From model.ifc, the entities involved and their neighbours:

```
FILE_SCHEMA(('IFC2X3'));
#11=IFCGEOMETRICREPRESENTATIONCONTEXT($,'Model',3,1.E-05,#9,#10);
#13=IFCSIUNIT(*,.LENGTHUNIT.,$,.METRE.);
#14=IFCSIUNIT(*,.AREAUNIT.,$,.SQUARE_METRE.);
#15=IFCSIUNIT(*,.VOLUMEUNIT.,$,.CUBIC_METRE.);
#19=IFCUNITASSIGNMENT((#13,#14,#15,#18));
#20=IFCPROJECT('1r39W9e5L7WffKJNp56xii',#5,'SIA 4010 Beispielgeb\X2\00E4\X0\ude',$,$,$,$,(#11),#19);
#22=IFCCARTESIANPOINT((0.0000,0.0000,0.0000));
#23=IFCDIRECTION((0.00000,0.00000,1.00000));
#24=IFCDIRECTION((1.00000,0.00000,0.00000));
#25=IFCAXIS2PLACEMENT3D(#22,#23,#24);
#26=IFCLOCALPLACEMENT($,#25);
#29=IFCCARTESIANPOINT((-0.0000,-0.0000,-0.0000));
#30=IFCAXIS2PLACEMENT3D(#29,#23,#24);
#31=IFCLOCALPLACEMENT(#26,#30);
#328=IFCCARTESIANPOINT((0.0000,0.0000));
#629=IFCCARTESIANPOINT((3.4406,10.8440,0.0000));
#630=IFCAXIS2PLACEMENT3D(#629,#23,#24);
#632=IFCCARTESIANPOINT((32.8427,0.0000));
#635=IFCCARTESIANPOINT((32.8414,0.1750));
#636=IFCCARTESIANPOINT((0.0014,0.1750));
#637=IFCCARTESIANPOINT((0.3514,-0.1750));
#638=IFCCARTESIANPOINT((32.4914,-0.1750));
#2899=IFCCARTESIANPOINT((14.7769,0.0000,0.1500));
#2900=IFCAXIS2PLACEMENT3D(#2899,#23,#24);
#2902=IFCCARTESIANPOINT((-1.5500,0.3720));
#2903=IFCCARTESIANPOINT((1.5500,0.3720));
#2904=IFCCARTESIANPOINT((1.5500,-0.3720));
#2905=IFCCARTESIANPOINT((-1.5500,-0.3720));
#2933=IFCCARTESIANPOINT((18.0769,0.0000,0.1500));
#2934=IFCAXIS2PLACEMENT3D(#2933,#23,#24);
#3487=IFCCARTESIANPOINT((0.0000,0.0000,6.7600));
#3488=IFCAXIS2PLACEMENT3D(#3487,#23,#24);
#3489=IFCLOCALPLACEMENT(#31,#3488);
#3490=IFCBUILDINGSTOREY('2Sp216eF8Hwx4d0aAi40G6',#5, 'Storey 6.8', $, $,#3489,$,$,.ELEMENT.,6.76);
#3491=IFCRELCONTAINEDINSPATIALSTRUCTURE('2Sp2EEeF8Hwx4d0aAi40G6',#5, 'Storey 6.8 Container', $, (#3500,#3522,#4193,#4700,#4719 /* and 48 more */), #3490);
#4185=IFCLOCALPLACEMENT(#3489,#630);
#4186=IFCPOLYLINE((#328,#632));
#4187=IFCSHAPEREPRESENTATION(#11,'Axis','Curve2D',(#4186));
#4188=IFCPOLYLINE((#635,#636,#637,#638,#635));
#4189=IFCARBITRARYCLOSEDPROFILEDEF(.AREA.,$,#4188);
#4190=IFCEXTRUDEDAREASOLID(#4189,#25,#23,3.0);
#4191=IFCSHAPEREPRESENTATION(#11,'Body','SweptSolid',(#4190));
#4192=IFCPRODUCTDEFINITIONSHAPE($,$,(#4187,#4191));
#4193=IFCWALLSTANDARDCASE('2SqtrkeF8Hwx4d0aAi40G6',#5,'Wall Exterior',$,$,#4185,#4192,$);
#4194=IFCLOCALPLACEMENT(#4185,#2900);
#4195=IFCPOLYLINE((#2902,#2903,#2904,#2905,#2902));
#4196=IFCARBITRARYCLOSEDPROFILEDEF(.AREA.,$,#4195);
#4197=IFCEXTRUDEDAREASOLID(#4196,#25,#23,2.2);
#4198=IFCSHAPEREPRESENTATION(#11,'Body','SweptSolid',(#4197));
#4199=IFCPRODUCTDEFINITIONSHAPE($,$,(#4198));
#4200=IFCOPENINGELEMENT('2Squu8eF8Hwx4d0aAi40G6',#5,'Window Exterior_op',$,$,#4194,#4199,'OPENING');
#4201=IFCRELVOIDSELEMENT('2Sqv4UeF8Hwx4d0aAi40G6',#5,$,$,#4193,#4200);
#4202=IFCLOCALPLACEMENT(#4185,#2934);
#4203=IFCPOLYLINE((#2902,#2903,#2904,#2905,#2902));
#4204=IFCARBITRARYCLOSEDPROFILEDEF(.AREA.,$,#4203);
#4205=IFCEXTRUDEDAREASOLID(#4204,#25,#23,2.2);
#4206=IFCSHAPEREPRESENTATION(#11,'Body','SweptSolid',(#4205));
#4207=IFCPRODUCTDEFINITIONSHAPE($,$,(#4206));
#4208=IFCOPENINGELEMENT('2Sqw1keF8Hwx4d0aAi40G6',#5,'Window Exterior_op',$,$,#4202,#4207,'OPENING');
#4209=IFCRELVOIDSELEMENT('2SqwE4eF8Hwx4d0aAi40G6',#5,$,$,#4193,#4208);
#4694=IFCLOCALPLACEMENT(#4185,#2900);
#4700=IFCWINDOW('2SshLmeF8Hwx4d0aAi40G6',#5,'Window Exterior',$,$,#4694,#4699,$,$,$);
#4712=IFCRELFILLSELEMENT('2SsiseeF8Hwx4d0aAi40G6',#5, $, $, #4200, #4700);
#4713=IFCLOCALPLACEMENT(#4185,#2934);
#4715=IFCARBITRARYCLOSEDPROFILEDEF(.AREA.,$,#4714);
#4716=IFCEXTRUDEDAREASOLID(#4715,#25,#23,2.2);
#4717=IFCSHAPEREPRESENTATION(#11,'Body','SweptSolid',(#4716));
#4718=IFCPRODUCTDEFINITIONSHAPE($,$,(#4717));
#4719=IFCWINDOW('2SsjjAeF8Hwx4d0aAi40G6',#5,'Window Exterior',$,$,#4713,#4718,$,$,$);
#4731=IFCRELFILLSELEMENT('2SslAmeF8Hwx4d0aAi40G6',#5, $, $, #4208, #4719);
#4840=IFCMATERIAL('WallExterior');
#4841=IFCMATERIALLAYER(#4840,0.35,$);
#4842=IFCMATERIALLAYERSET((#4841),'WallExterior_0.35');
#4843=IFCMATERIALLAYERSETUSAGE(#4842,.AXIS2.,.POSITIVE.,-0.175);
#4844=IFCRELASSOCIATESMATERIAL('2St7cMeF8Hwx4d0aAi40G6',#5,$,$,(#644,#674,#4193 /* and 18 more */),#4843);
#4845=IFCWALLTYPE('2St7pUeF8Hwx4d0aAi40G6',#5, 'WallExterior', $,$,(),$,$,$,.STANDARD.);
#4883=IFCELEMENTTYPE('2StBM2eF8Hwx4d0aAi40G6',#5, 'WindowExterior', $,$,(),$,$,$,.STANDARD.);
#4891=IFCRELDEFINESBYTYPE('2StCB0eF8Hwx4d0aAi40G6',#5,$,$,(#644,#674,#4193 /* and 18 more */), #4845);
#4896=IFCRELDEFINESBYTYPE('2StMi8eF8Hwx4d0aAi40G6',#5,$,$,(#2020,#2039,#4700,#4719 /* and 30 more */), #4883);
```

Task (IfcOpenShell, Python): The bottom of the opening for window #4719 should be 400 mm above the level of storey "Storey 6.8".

```python
import numpy as np
import ifcopenshell
import ifcopenshell.api.geometry
import ifcopenshell.geom
import ifcopenshell.util.element
import ifcopenshell.util.placement
import ifcopenshell.util.shape
import ifcopenshell.util.unit

model = ifcopenshell.open("model.ifc")
unit_scale = ifcopenshell.util.unit.calculate_unit_scale(model)

window = model.by_guid("2SsjjAeF8Hwx4d0aAi40G6")
opening = window.FillsVoids[0].RelatingOpeningElement
storey = ifcopenshell.util.element.get_container(window, ifc_class="IfcBuildingStorey")
level = ifcopenshell.util.placement.get_local_placement(storey.ObjectPlacement)[2, 3]

# The opening's origin need not be at the sill, so measure its lowest point.
shape = ifcopenshell.geom.create_shape(ifcopenshell.geom.settings(), opening)
bottom = ifcopenshell.util.shape.get_shape_bottom_elevation(shape, shape.geometry) / unit_scale
dz = level + 0.4 / unit_scale - bottom

shift = np.array([0.0, 0.0, dz])
# The window is not placed relative to its opening, so move both.
for product in (opening, window):
    matrix = ifcopenshell.util.placement.get_local_placement(product.ObjectPlacement)
    matrix[:3, 3] += shift
    ifcopenshell.api.geometry.edit_object_placement(model, product=product, matrix=matrix, is_si=False)

print(f"moved by {dz * unit_scale:+.3f} m")

model.write("model-out.ifc")
```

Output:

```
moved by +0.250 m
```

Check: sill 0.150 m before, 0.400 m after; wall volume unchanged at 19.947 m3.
